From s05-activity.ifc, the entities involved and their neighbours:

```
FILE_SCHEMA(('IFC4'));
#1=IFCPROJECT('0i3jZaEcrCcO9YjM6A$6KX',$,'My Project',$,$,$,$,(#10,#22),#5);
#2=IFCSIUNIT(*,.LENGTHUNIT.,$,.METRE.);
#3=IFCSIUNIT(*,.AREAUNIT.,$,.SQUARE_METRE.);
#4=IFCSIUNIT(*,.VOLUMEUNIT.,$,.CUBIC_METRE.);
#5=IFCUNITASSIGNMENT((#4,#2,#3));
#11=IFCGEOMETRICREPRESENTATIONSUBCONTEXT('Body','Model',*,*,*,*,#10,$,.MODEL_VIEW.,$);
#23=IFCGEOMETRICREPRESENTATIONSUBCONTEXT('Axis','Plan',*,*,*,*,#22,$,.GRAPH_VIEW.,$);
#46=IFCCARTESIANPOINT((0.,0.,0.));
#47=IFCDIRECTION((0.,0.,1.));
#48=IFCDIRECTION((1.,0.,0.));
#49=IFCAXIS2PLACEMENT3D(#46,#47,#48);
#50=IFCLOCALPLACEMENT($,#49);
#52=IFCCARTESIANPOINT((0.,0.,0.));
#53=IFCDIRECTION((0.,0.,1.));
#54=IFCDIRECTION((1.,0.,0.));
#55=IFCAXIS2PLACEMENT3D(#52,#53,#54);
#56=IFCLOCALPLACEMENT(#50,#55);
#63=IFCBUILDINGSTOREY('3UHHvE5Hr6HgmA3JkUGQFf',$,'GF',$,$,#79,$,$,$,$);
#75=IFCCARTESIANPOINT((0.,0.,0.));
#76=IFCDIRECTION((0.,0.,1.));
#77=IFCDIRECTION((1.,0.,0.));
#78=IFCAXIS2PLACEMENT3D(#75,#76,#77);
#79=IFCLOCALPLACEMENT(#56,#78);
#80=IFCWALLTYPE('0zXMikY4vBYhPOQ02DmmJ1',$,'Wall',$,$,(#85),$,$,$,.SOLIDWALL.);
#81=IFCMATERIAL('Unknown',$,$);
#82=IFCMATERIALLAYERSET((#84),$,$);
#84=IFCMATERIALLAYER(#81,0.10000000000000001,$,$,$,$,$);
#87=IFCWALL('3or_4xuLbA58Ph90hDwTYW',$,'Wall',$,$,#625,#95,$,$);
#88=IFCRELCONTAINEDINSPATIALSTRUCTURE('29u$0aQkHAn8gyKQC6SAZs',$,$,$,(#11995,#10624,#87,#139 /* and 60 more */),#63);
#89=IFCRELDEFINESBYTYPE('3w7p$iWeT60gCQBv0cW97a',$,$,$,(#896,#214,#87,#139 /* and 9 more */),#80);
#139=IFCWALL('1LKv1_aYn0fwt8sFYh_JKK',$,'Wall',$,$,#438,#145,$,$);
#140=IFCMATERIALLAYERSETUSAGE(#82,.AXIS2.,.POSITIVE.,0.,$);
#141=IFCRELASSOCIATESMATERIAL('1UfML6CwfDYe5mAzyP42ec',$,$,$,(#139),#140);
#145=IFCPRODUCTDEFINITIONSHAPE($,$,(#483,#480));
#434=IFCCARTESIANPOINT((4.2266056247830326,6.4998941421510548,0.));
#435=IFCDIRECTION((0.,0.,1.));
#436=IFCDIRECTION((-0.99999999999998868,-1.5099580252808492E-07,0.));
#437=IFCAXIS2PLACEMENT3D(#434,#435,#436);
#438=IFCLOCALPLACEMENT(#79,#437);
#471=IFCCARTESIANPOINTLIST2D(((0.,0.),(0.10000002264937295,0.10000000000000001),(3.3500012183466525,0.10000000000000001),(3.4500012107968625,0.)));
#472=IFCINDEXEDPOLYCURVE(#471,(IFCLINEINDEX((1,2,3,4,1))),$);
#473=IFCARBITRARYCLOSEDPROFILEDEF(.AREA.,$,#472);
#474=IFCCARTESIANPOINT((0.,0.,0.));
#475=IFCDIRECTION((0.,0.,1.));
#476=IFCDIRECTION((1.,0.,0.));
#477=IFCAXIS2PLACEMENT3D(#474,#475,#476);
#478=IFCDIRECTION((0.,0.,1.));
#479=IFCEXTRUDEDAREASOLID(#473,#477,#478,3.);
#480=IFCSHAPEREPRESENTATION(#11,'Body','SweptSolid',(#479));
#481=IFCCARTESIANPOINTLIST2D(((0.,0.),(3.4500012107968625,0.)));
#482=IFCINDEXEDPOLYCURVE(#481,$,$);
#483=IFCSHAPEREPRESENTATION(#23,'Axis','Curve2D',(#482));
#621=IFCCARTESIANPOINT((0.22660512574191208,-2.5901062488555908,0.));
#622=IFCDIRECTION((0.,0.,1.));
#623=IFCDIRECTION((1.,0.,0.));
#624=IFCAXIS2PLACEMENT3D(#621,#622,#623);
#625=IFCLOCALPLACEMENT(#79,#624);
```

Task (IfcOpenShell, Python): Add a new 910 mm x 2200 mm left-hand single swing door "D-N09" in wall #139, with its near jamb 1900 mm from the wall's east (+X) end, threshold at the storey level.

```python
import numpy as np
import ifcopenshell
import ifcopenshell.api.feature
import ifcopenshell.api.geometry
import ifcopenshell.api.root
import ifcopenshell.api.spatial
import ifcopenshell.geom
import ifcopenshell.util.element
import ifcopenshell.util.placement
import ifcopenshell.util.representation
import ifcopenshell.util.shape
import ifcopenshell.util.unit

model = ifcopenshell.open("s05-activity.ifc")
unit_scale = ifcopenshell.util.unit.calculate_unit_scale(model)
settings = ifcopenshell.geom.settings()


def volume(element):
    """Net volume in cubic metres, openings subtracted."""
    shape = ifcopenshell.geom.create_shape(settings, element)
    return ifcopenshell.util.shape.get_volume(shape.geometry)


wall = model.by_guid("1LKv1_aYn0fwt8sFYh_JKK")
storey = ifcopenshell.util.element.get_container(wall, ifc_class="IfcBuildingStorey")
context = ifcopenshell.util.representation.get_context(model, "Model", "Body", "MODEL_VIEW")
before = volume(wall)

width, height, from_end, sill = 0.91, 2.2, 1.9, 0.0  # metres

# The wall runs along its own X axis, and the end named is its -X end.
wall_shape = ifcopenshell.geom.create_shape(settings, wall)
x, y, z = ifcopenshell.util.shape.get_vertices(wall_shape.geometry).T
start = x.min() + from_end
face, thickness = float(y.min()), float(y.max() - y.min())
wall_matrix = ifcopenshell.util.placement.get_local_placement(wall.ObjectPlacement)
level = ifcopenshell.util.placement.get_local_placement(storey.ObjectPlacement)[2, 3]


def in_wall(x, y):
    """Placement at x, y metres in the wall's axes, at sill height."""
    matrix = wall_matrix.copy()
    matrix[:, 3] = wall_matrix @ np.array([x / unit_scale, y / unit_scale, 0.0, 1.0])
    matrix[2, 3] = level + sill / unit_scale
    return matrix


# Opening: a box that overshoots both wall faces by 50 mm.
opening = ifcopenshell.api.root.create_entity(model, ifc_class="IfcOpeningElement", predefined_type="OPENING")
box = ifcopenshell.api.geometry.add_wall_representation(
    model, context=context, length=width, height=height, thickness=thickness + 0.1
)
ifcopenshell.api.geometry.assign_representation(model, product=opening, representation=box)
ifcopenshell.api.geometry.edit_object_placement(model, product=opening, matrix=in_wall(start, face - 0.05), is_si=False)
ifcopenshell.api.feature.add_feature(model, feature=opening, element=wall)

door = ifcopenshell.api.root.create_entity(model, ifc_class="IfcDoor", name="D-N09", predefined_type="DOOR")
door.OverallWidth, door.OverallHeight = width / unit_scale, height / unit_scale
door.OperationType = "SINGLE_SWING_LEFT"
body = ifcopenshell.api.geometry.add_door_representation(
    model,
    context=context,
    overall_width=door.OverallWidth,
    overall_height=door.OverallHeight,
    operation_type="SINGLE_SWING_LEFT",
    lining_properties={"LiningDepth": thickness / unit_scale, "ThresholdDepth": thickness / unit_scale},
)
ifcopenshell.api.geometry.assign_representation(model, product=door, representation=body)
ifcopenshell.api.spatial.assign_container(model, products=[door], relating_structure=storey)
ifcopenshell.api.feature.add_filling(model, opening=opening, element=door)

# The lining spans the wall, so the door starts at the wall face.
ifcopenshell.api.geometry.edit_object_placement(model, product=door, matrix=in_wall(start, face), is_si=False)

after = volume(wall)

print(f"wall volume {before:.3f} -> {after:.3f} m3")

model.write("s05-activity_rev.ifc")
```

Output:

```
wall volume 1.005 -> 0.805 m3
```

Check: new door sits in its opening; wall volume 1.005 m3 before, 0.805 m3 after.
